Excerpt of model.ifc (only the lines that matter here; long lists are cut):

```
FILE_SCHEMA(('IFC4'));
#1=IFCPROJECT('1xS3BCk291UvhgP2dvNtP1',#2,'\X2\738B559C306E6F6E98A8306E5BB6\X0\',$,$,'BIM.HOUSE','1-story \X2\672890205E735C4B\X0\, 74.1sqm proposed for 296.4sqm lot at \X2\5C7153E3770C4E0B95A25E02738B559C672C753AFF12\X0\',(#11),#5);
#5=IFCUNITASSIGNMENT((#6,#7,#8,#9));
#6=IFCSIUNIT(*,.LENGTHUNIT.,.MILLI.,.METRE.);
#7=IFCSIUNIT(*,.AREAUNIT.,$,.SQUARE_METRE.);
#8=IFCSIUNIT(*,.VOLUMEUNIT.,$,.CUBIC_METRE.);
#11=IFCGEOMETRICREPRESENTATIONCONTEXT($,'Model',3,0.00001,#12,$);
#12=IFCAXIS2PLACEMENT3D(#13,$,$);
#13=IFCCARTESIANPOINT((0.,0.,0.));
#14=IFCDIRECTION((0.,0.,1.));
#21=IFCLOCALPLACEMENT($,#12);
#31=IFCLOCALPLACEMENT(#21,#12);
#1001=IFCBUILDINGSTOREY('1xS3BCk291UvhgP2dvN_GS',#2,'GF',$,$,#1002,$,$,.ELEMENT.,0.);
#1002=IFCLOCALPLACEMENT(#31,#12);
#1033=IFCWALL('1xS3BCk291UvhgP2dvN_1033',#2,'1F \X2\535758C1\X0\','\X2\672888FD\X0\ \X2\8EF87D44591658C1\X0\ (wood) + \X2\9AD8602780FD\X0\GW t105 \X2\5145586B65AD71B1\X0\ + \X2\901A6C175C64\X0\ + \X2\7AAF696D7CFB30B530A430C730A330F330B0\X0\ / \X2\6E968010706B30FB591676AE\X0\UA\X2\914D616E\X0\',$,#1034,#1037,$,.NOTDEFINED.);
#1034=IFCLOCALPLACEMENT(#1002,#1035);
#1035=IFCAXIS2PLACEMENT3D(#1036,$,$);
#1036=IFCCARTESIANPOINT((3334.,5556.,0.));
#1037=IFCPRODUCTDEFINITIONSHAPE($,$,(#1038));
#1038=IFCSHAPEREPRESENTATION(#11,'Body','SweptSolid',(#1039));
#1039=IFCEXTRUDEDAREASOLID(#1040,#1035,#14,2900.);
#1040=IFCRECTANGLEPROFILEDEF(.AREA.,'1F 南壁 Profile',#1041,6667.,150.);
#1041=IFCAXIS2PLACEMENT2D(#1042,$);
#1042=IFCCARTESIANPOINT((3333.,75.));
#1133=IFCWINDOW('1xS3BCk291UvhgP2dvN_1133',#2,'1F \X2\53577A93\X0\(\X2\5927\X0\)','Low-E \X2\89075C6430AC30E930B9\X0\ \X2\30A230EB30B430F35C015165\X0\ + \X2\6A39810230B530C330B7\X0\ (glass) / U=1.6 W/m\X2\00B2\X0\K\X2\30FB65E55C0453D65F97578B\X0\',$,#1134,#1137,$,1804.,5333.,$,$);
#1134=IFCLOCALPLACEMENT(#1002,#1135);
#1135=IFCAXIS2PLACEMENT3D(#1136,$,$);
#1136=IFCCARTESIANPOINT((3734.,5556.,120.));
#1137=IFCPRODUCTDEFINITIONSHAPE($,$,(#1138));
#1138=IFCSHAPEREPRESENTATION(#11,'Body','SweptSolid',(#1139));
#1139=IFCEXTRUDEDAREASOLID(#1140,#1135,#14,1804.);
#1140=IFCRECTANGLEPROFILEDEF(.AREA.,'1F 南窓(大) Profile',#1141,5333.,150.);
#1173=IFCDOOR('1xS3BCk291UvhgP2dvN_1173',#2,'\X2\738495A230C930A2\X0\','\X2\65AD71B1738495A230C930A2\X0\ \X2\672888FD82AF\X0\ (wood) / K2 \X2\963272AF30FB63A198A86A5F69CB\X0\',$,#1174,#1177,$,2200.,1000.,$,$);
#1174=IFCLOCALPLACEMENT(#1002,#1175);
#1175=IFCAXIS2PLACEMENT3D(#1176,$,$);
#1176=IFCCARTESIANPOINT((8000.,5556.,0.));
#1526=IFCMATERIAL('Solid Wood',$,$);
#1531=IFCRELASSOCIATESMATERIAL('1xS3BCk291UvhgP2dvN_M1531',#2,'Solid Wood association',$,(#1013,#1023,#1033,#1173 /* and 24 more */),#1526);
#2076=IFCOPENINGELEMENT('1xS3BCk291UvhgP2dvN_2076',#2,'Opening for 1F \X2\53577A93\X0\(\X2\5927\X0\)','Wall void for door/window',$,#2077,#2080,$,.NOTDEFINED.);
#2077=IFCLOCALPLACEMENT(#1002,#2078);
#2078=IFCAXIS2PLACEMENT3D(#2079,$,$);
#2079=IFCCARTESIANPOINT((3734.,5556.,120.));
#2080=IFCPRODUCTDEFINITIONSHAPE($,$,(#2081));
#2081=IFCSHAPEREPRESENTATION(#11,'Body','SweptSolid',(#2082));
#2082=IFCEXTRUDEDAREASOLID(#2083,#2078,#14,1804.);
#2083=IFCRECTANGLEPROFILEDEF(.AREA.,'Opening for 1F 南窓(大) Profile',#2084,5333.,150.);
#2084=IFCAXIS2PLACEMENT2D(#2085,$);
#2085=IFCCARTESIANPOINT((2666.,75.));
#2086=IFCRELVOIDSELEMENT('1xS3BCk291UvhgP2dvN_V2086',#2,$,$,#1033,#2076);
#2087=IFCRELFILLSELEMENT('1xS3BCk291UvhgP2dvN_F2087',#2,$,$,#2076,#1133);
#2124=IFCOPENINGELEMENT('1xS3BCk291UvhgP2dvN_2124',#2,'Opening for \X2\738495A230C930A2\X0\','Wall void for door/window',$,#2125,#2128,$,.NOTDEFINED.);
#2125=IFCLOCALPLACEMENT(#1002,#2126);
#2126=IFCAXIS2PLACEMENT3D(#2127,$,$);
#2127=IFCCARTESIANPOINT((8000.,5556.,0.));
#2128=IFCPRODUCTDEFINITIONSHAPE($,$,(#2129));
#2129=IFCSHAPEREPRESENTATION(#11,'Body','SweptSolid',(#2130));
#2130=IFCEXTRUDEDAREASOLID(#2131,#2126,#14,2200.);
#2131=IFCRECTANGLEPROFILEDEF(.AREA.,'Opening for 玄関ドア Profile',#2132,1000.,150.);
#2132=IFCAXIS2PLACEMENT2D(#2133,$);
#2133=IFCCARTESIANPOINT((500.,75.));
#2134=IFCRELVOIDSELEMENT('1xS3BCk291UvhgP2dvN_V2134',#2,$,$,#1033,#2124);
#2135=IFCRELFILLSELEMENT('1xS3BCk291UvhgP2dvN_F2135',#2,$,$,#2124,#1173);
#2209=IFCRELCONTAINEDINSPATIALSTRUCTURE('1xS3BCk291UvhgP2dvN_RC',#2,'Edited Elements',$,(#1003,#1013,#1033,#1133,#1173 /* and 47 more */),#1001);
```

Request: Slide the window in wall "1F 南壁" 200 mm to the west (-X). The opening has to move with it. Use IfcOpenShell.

```python
import ifcopenshell
import ifcopenshell.api.geometry
import ifcopenshell.util.placement
import ifcopenshell.util.unit

model = ifcopenshell.open("model.ifc")
unit_scale = ifcopenshell.util.unit.calculate_unit_scale(model)

window = model.by_guid("1xS3BCk291UvhgP2dvN_1133")
opening = window.FillsVoids[0].RelatingOpeningElement
wall = opening.VoidsElements[0].RelatingBuildingElement

wall_matrix = ifcopenshell.util.placement.get_local_placement(wall.ObjectPlacement)
shift = wall_matrix[:3, 0] * -0.2 / unit_scale
before = ifcopenshell.util.placement.get_local_placement(window.ObjectPlacement)[:3, 3].copy()

# The window is not placed relative to its opening, so move both.
for product in (opening, window):
    matrix = ifcopenshell.util.placement.get_local_placement(product.ObjectPlacement)
    matrix[:3, 3] += shift
    ifcopenshell.api.geometry.edit_object_placement(model, product=product, matrix=matrix, is_si=False)

after = ifcopenshell.util.placement.get_local_placement(window.ObjectPlacement)[:3, 3]
print("window moved by", (after - before).round(3) + 0.0)

model.write("model_v2.ifc")
```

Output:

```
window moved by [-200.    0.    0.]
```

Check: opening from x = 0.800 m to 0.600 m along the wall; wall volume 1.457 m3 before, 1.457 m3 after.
